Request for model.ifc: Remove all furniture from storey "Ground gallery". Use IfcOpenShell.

First a look at what the model holds.

```python
import ifcopenshell
import ifcopenshell.util.element

model = ifcopenshell.open("model.ifc")
print(model.schema)
storey = next(s for s in model.by_type("IfcBuildingStorey") if s.Name == "Ground gallery")
furniture = [e for e in ifcopenshell.util.element.get_decomposition(storey) if e.is_a("IfcFurnishingElement")]
seen = {}
for e in furniture:
    element_type = ifcopenshell.util.element.get_type(e)
    name = element_type.Name if element_type not in (None, e) else None
    seen[name] = seen.get(name, 0) + 1
for name, count in sorted(seen.items(), key=str):
    print(count, "x", name)
```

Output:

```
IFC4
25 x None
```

```python
import ifcopenshell
import ifcopenshell.api.root
import ifcopenshell.util.element

model = ifcopenshell.open("model.ifc")

storey = next(s for s in model.by_type("IfcBuildingStorey") if s.Name == "Ground gallery")
furniture = [e for e in ifcopenshell.util.element.get_decomposition(storey) if e.is_a("IfcFurnishingElement")]

for e in furniture:
    ifcopenshell.api.root.remove_product(model, product=e)
print(len(furniture), "removed")

model.write("model_updated.ifc")
```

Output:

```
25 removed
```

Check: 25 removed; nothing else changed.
